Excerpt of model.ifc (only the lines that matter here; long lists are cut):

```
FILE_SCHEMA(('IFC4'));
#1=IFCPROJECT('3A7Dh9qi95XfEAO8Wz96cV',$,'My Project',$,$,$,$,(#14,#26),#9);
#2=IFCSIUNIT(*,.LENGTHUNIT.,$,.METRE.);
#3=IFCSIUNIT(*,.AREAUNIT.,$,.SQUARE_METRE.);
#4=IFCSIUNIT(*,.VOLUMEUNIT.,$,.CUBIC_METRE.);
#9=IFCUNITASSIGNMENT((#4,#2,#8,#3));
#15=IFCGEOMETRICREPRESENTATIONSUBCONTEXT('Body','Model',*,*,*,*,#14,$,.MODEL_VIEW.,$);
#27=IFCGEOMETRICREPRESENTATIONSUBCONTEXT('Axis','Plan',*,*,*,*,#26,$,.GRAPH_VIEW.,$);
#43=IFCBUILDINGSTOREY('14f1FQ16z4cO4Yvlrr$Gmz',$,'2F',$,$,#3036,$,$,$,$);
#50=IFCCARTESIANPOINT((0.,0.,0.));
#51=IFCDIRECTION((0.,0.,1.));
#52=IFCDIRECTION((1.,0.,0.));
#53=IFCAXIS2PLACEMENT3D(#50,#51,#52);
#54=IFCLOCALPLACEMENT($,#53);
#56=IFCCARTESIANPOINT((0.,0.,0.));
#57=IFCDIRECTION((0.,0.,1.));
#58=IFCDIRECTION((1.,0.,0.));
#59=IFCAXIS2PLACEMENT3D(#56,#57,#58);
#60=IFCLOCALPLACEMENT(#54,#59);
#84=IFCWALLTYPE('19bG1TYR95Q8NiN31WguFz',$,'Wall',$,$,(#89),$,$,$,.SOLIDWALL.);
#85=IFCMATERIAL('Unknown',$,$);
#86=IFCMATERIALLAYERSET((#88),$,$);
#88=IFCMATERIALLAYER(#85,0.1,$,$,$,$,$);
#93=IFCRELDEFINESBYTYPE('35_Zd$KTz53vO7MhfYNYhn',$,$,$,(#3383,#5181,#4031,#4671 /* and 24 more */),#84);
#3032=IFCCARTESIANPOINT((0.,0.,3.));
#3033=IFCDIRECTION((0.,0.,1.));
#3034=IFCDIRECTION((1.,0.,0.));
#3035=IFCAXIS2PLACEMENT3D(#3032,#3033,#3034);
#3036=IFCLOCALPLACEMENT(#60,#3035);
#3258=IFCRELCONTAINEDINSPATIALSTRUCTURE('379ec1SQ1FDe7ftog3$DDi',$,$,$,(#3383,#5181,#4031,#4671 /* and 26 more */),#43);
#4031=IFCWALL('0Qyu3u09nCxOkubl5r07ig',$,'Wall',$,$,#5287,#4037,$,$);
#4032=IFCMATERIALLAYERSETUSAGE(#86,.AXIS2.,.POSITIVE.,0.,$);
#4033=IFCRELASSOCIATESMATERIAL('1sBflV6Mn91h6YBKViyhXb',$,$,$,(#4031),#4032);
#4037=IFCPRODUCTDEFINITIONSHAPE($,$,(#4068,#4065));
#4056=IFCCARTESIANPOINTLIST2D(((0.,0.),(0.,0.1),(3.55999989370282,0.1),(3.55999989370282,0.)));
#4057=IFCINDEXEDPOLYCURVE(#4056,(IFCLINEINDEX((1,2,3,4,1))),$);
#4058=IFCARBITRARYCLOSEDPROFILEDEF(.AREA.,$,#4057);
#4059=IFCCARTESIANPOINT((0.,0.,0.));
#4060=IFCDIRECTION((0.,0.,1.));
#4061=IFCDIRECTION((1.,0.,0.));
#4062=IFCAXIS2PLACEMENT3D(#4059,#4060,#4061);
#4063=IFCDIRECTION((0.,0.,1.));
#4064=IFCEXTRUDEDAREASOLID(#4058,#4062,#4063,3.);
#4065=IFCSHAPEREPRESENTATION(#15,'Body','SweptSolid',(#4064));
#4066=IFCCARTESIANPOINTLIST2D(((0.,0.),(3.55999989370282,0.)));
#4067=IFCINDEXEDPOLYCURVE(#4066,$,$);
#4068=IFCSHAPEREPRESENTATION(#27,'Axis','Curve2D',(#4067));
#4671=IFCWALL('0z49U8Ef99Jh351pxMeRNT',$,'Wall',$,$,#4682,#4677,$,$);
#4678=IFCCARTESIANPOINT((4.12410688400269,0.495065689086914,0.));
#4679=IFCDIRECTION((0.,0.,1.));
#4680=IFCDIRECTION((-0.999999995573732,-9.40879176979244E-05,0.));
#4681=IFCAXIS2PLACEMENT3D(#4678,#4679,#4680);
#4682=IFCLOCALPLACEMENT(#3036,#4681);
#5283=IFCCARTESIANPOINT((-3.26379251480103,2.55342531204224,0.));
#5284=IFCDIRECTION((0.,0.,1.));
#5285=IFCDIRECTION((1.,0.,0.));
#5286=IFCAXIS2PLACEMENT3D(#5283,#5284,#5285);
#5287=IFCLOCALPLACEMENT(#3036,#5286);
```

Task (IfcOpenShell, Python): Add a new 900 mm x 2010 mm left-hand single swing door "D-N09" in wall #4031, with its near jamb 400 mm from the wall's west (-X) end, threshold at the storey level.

```python
import numpy as np
import ifcopenshell
import ifcopenshell.api.feature
import ifcopenshell.api.geometry
import ifcopenshell.api.root
import ifcopenshell.api.spatial
import ifcopenshell.geom
import ifcopenshell.util.element
import ifcopenshell.util.placement
import ifcopenshell.util.representation
import ifcopenshell.util.shape
import ifcopenshell.util.unit

model = ifcopenshell.open("model.ifc")
unit_scale = ifcopenshell.util.unit.calculate_unit_scale(model)
settings = ifcopenshell.geom.settings()


def volume(element):
    """Net volume in cubic metres, openings subtracted."""
    shape = ifcopenshell.geom.create_shape(settings, element)
    return ifcopenshell.util.shape.get_volume(shape.geometry)


wall = model.by_guid("0Qyu3u09nCxOkubl5r07ig")
storey = ifcopenshell.util.element.get_container(wall, ifc_class="IfcBuildingStorey")
context = ifcopenshell.util.representation.get_context(model, "Model", "Body", "MODEL_VIEW")
before = volume(wall)

width, height, from_end, sill = 0.9, 2.01, 0.4, 0.0  # metres

# The wall runs along its own X axis, and the end named is its -X end.
wall_shape = ifcopenshell.geom.create_shape(settings, wall)
x, y, z = ifcopenshell.util.shape.get_vertices(wall_shape.geometry).T
start = x.min() + from_end
face, thickness = float(y.min()), float(y.max() - y.min())
wall_matrix = ifcopenshell.util.placement.get_local_placement(wall.ObjectPlacement)
level = ifcopenshell.util.placement.get_local_placement(storey.ObjectPlacement)[2, 3]


def in_wall(x, y):
    """Placement at x, y metres in the wall's axes, at sill height."""
    matrix = wall_matrix.copy()
    matrix[:, 3] = wall_matrix @ np.array([x / unit_scale, y / unit_scale, 0.0, 1.0])
    matrix[2, 3] = level + sill / unit_scale
    return matrix


# Opening: a box that overshoots both wall faces by 50 mm.
opening = ifcopenshell.api.root.create_entity(model, ifc_class="IfcOpeningElement", predefined_type="OPENING")
box = ifcopenshell.api.geometry.add_wall_representation(
    model, context=context, length=width, height=height, thickness=thickness + 0.1
)
ifcopenshell.api.geometry.assign_representation(model, product=opening, representation=box)
ifcopenshell.api.geometry.edit_object_placement(model, product=opening, matrix=in_wall(start, face - 0.05), is_si=False)
ifcopenshell.api.feature.add_feature(model, feature=opening, element=wall)

door = ifcopenshell.api.root.create_entity(model, ifc_class="IfcDoor", name="D-N09", predefined_type="DOOR")
door.OverallWidth, door.OverallHeight = width / unit_scale, height / unit_scale
door.OperationType = "SINGLE_SWING_LEFT"
body = ifcopenshell.api.geometry.add_door_representation(
    model,
    context=context,
    overall_width=door.OverallWidth,
    overall_height=door.OverallHeight,
    operation_type="SINGLE_SWING_LEFT",
    lining_properties={"LiningDepth": thickness / unit_scale, "ThresholdDepth": thickness / unit_scale},
)
ifcopenshell.api.geometry.assign_representation(model, product=door, representation=body)
ifcopenshell.api.spatial.assign_container(model, products=[door], relating_structure=storey)
ifcopenshell.api.feature.add_filling(model, opening=opening, element=door)

# The lining spans the wall, so the door starts at the wall face.
ifcopenshell.api.geometry.edit_object_placement(model, product=door, matrix=in_wall(start, face), is_si=False)

after = volume(wall)

print(f"wall volume {before:.3f} -> {after:.3f} m3")

model.write("model_v2.ifc")
```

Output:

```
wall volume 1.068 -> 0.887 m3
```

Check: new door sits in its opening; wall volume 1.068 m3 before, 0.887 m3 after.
